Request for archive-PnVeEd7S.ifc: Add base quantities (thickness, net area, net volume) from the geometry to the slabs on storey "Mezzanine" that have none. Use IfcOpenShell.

First a look at what the model holds.

```python
import ifcopenshell
import ifcopenshell.util.element
import ifcopenshell.util.unit

model = ifcopenshell.open("archive-PnVeEd7S.ifc")
print(model.schema)
for unit_type in ("LENGTHUNIT", "AREAUNIT", "VOLUMEUNIT"):
    print(unit_type, ifcopenshell.util.unit.calculate_unit_scale(model, unit_type))
storey = next(s for s in model.by_type("IfcBuildingStorey") if s.Name == "Mezzanine")
slabs = [e for e in ifcopenshell.util.element.get_decomposition(storey) if e.is_a("IfcSlab")]
for e in sorted(slabs, key=lambda e: e.id()):
    print(e.id(), e.is_a(), e.Name, list(ifcopenshell.util.element.get_psets(e, qtos_only=True)), sep=" | ")
```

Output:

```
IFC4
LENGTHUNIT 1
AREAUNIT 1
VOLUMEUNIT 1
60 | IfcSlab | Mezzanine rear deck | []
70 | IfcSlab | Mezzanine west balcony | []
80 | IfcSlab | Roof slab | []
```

```python
import ifcopenshell
import ifcopenshell.api.pset
import ifcopenshell.geom
import ifcopenshell.util.element
import ifcopenshell.util.shape
import ifcopenshell.util.unit

model = ifcopenshell.open("archive-PnVeEd7S.ifc")
unit_scale = ifcopenshell.util.unit.calculate_unit_scale(model)
area_scale = ifcopenshell.util.unit.calculate_unit_scale(model, "AREAUNIT")
volume_scale = ifcopenshell.util.unit.calculate_unit_scale(model, "VOLUMEUNIT")
settings = ifcopenshell.geom.settings()

storey = next(s for s in model.by_type("IfcBuildingStorey") if s.Name == "Mezzanine")
slabs = [e for e in ifcopenshell.util.element.get_decomposition(storey) if e.is_a("IfcSlab")]

for e in sorted(slabs, key=lambda e: e.id()):
    if ifcopenshell.util.element.get_psets(e, qtos_only=True, should_inherit=False):
        continue
    # Geometry comes back in metres, in the element's own axes.
    shape = ifcopenshell.geom.create_shape(settings, e)
    values = {
        "Width": ifcopenshell.util.shape.get_z(shape.geometry) / unit_scale,
        "NetArea": ifcopenshell.util.shape.get_footprint_area(shape.geometry) / area_scale,
        "NetVolume": ifcopenshell.util.shape.get_volume(shape.geometry) / volume_scale,
    }
    qto = ifcopenshell.api.pset.add_qto(model, product=e, name="Qto_SlabBaseQuantities")
    ifcopenshell.api.pset.edit_qto(model, qto=qto, properties=values)
    print(e.id(), {k: round(v, 3) for k, v in values.items()})

model.write("archive-PnVeEd7S_v2.ifc")
```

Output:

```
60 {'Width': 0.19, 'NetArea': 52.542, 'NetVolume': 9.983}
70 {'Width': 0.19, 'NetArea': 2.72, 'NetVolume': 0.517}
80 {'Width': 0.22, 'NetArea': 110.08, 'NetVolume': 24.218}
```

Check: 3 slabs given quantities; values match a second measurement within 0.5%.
